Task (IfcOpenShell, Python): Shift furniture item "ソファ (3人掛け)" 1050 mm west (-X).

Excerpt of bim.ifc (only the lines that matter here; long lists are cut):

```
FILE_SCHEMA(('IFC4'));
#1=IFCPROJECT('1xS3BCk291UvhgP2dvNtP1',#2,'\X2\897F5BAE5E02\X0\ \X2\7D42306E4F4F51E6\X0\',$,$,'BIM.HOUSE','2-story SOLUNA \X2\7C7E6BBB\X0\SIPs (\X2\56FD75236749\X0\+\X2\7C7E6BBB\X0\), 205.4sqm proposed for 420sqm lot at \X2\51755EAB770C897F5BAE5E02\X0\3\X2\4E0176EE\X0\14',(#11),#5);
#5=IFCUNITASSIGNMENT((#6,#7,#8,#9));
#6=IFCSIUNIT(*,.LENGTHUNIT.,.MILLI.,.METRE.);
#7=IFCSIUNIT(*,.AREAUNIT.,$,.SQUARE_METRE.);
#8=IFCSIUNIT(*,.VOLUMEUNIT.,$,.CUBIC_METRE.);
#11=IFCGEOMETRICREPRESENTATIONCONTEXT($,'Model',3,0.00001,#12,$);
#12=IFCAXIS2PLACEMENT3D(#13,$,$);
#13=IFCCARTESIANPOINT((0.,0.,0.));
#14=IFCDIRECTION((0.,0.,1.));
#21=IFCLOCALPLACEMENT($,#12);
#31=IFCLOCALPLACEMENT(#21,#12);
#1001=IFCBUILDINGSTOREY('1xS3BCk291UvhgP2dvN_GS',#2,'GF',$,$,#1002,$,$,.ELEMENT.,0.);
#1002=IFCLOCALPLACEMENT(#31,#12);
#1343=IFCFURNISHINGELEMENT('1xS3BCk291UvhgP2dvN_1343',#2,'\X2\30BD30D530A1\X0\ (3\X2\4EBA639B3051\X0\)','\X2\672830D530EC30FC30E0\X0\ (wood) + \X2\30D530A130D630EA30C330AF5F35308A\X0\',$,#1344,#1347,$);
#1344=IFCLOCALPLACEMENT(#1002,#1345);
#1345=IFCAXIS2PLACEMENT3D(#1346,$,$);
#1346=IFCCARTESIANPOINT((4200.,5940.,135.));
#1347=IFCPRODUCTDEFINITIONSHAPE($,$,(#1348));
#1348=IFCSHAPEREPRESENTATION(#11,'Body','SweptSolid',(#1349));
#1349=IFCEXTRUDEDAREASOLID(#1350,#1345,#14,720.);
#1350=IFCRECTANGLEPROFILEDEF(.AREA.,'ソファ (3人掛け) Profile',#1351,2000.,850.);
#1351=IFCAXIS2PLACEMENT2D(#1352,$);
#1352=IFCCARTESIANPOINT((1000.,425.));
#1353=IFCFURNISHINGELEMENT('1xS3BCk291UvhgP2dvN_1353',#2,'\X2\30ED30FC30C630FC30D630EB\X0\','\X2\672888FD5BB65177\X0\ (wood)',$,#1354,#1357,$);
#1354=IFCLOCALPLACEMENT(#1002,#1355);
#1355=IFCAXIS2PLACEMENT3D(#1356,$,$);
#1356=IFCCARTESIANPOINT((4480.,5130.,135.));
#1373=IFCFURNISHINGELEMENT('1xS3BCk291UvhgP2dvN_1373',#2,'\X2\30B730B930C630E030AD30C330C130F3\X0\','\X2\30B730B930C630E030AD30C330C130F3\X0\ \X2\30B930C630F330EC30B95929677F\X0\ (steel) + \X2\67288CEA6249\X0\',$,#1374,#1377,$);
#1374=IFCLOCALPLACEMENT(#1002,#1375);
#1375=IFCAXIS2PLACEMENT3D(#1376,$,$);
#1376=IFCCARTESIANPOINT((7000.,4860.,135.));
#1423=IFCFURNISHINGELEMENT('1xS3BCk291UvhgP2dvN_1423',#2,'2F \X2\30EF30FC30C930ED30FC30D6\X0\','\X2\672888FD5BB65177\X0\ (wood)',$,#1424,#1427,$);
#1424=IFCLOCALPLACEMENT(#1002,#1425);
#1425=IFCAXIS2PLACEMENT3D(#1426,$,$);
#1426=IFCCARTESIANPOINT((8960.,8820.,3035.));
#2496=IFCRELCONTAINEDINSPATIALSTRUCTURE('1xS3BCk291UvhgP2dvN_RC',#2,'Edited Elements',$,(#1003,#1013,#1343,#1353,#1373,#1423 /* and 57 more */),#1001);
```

```python
import ifcopenshell
import ifcopenshell.api.geometry
import ifcopenshell.util.placement
import ifcopenshell.util.unit

model = ifcopenshell.open("bim.ifc")
unit_scale = ifcopenshell.util.unit.calculate_unit_scale(model)

item = model.by_guid("1xS3BCk291UvhgP2dvN_1343")
matrix = ifcopenshell.util.placement.get_local_placement(item.ObjectPlacement)
matrix[0, 3] -= 1.05 / unit_scale
ifcopenshell.api.geometry.edit_object_placement(model, product=item, matrix=matrix, is_si=False)

print(ifcopenshell.util.placement.get_local_placement(item.ObjectPlacement).round(3) + 0.0)

model.write("bim_v2.ifc")
```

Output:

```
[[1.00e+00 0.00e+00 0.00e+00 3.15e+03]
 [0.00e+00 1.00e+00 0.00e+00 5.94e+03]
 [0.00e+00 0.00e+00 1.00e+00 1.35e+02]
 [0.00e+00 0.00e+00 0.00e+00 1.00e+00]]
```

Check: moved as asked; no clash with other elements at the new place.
